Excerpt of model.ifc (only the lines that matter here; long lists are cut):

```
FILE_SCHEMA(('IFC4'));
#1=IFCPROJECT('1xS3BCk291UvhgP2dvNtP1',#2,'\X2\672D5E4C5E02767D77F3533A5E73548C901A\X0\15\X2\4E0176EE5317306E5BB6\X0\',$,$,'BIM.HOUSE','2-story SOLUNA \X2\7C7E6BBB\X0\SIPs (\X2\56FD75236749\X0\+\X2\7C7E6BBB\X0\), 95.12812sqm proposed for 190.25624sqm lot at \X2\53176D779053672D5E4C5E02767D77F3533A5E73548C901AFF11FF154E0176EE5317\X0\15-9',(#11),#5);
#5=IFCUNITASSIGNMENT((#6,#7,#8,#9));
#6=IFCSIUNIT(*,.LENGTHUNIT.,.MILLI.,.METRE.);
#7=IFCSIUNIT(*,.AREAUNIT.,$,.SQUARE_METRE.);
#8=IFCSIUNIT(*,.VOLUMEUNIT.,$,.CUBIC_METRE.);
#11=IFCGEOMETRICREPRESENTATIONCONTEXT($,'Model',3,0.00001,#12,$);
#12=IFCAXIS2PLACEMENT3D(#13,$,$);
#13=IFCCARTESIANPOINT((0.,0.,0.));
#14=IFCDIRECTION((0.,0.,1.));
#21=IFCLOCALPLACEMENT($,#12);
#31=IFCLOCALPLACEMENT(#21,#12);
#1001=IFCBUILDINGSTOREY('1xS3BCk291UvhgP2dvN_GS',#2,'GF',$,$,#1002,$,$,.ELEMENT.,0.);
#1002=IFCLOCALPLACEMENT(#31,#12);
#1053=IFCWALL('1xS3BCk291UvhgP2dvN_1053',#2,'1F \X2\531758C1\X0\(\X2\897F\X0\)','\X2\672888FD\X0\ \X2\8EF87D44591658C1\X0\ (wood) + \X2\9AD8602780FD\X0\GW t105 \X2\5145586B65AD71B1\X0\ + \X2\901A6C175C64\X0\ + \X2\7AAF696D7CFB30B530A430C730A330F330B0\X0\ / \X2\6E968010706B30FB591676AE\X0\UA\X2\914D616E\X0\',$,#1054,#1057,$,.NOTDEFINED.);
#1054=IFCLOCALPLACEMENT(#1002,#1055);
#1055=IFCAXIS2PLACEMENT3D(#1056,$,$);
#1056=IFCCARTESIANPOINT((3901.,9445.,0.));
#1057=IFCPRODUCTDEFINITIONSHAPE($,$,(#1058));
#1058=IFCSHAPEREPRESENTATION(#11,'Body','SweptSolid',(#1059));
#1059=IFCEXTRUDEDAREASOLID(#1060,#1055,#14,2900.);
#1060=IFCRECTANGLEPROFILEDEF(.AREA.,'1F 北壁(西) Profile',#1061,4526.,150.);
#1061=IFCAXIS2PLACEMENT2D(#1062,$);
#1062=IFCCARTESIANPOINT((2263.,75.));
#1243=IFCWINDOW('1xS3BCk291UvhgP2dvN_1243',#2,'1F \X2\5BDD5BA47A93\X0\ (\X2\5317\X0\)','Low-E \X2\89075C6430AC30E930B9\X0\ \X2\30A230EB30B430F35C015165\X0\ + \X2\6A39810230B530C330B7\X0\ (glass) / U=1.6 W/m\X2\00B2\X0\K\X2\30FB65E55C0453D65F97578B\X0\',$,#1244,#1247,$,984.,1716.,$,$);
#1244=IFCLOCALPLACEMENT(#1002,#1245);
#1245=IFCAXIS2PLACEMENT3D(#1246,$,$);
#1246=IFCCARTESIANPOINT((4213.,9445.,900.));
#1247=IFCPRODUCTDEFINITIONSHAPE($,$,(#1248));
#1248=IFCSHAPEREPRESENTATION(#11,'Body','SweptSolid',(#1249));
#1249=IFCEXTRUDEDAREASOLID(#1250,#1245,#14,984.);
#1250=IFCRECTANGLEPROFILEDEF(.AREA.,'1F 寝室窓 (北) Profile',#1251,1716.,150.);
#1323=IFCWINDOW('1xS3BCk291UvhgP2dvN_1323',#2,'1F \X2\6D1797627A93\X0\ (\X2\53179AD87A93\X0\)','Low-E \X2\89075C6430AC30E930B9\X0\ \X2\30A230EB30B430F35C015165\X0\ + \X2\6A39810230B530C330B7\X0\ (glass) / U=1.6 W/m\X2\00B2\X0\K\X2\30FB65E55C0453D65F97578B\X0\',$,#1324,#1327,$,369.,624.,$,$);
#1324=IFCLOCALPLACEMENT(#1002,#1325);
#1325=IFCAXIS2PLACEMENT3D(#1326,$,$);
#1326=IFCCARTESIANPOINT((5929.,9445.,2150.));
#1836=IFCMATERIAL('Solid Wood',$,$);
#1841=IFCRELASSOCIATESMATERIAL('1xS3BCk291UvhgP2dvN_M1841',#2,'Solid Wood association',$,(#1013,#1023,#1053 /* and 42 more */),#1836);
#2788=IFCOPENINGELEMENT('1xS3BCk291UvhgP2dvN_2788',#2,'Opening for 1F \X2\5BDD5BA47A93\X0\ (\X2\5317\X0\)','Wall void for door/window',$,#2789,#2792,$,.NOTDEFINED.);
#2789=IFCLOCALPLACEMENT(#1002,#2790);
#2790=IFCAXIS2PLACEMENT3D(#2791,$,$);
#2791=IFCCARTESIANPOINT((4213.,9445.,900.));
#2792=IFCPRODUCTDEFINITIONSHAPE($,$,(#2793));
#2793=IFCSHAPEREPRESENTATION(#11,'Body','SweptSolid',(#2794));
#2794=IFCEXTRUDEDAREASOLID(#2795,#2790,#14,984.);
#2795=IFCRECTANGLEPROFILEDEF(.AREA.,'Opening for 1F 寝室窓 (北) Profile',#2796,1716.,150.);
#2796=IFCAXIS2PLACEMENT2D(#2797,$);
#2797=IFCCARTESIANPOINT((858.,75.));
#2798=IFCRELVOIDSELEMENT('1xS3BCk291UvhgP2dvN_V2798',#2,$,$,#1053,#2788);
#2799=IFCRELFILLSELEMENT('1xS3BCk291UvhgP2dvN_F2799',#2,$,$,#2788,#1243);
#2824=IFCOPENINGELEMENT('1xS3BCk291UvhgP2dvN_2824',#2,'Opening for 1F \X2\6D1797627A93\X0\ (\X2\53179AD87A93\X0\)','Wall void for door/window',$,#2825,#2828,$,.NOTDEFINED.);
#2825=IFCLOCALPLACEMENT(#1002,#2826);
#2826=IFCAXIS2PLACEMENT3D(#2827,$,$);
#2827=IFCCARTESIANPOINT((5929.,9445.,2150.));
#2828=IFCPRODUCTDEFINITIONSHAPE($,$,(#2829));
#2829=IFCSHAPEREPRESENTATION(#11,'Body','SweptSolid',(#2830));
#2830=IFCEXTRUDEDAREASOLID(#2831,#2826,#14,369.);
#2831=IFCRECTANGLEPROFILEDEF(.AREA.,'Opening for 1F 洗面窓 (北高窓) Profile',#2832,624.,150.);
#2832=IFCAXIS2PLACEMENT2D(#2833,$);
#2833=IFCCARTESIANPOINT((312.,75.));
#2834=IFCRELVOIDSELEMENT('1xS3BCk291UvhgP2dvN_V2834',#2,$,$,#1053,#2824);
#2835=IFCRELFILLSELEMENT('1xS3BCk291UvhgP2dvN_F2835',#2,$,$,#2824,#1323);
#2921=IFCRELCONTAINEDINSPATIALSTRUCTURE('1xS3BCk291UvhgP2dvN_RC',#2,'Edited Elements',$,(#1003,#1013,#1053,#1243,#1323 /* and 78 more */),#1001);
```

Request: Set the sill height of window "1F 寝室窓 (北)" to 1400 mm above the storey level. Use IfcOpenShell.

```python
import numpy as np
import ifcopenshell
import ifcopenshell.api.geometry
import ifcopenshell.geom
import ifcopenshell.util.element
import ifcopenshell.util.placement
import ifcopenshell.util.shape
import ifcopenshell.util.unit

model = ifcopenshell.open("model.ifc")
unit_scale = ifcopenshell.util.unit.calculate_unit_scale(model)

window = model.by_id(1243)
opening = window.FillsVoids[0].RelatingOpeningElement
storey = ifcopenshell.util.element.get_container(window, ifc_class="IfcBuildingStorey")
level = ifcopenshell.util.placement.get_local_placement(storey.ObjectPlacement)[2, 3]

# The opening's origin need not be at the sill, so measure its lowest point.
shape = ifcopenshell.geom.create_shape(ifcopenshell.geom.settings(), opening)
bottom = ifcopenshell.util.shape.get_shape_bottom_elevation(shape, shape.geometry) / unit_scale
dz = level + 1400.0 - bottom

shift = np.array([0.0, 0.0, dz])
# The window is not placed relative to its opening, so move both.
for product in (opening, window):
    matrix = ifcopenshell.util.placement.get_local_placement(product.ObjectPlacement)
    matrix[:3, 3] += shift
    ifcopenshell.api.geometry.edit_object_placement(model, product=product, matrix=matrix, is_si=False)

print(f"moved by {dz * unit_scale:+.3f} m")

model.write("model_rev.ifc")
```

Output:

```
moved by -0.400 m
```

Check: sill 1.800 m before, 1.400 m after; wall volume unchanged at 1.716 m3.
